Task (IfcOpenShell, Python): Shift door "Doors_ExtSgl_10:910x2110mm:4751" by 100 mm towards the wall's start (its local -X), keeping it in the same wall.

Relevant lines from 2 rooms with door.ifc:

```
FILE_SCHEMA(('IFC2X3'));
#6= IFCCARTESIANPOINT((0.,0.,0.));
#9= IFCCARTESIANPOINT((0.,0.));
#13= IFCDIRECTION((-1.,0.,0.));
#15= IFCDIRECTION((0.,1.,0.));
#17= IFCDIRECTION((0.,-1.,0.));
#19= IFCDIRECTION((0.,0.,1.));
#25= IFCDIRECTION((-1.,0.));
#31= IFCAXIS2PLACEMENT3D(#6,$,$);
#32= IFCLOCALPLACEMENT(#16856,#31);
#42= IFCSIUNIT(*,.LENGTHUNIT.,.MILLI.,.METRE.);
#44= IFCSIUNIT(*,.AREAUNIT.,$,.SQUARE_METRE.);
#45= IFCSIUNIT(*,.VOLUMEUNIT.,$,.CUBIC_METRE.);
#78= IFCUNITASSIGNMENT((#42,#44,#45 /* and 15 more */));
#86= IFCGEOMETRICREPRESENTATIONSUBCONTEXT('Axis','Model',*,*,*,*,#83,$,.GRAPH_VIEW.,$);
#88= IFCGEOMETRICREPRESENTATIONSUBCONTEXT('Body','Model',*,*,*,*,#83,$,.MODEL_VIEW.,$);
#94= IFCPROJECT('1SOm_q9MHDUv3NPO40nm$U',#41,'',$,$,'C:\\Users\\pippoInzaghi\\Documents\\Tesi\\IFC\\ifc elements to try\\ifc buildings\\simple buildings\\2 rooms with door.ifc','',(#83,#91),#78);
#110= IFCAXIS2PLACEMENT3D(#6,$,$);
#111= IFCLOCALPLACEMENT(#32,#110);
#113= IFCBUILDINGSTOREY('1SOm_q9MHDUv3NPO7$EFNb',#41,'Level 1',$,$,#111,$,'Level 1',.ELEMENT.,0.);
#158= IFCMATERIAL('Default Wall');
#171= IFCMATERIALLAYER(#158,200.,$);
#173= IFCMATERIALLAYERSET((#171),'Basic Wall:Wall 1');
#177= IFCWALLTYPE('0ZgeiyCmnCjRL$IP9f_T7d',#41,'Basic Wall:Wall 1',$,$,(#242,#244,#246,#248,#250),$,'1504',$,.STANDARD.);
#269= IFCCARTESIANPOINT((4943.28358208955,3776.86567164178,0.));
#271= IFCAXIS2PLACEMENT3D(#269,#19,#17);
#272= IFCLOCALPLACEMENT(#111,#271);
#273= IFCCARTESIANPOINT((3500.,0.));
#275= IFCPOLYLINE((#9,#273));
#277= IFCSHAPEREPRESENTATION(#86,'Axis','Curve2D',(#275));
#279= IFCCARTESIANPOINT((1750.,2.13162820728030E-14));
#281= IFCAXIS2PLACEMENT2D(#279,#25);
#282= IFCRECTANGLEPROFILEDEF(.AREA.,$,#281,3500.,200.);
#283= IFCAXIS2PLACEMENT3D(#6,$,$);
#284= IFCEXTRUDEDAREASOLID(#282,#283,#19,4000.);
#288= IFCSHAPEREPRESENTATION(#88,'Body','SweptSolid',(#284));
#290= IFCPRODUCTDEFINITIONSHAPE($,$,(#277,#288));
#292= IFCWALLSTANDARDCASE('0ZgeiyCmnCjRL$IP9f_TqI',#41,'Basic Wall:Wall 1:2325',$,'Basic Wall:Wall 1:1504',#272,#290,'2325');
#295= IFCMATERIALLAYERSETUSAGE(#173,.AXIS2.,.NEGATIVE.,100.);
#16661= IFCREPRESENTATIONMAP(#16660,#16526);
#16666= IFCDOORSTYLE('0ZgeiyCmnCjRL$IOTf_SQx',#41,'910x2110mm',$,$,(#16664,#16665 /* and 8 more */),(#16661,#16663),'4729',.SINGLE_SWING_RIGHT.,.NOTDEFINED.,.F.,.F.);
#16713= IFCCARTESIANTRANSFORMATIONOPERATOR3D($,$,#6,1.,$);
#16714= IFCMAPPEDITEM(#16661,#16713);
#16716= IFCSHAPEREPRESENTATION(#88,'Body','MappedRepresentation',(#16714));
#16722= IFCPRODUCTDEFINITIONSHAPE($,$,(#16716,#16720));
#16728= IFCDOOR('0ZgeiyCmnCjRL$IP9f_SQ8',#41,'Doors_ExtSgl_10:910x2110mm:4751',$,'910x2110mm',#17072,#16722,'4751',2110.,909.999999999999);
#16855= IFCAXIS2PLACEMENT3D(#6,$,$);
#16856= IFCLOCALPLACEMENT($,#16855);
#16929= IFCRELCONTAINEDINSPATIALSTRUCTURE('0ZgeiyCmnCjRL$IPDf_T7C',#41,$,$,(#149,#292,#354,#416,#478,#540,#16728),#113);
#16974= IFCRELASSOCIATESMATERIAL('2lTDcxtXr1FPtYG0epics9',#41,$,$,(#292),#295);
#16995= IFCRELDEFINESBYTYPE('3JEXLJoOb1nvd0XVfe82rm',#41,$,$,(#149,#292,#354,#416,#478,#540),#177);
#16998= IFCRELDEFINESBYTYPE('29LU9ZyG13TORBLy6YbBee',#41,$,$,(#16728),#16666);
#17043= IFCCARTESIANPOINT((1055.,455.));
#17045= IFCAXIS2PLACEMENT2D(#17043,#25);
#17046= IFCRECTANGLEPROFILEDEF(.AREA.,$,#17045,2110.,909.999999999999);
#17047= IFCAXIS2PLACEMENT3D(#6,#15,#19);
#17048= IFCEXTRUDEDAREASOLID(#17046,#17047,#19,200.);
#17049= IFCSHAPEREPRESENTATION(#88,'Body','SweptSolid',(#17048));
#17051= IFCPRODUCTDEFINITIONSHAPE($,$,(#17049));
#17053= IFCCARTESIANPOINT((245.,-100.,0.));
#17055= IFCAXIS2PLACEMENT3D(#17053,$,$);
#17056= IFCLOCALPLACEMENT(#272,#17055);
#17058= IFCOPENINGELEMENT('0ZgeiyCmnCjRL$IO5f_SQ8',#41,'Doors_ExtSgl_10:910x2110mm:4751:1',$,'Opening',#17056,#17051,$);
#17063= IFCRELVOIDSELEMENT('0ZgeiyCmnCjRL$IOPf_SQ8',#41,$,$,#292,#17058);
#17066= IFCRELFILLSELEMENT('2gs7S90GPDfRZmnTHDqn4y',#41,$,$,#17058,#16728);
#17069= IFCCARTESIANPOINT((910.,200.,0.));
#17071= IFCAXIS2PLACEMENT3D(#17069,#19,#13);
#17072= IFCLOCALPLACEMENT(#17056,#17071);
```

```python
import ifcopenshell
import ifcopenshell.api.geometry
import ifcopenshell.util.placement
import ifcopenshell.util.unit

model = ifcopenshell.open("2 rooms with door.ifc")
unit_scale = ifcopenshell.util.unit.calculate_unit_scale(model)

door = model.by_id(16728)
opening = door.FillsVoids[0].RelatingOpeningElement
wall = opening.VoidsElements[0].RelatingBuildingElement

wall_matrix = ifcopenshell.util.placement.get_local_placement(wall.ObjectPlacement)
shift = wall_matrix[:3, 0] * -0.1 / unit_scale
before = ifcopenshell.util.placement.get_local_placement(door.ObjectPlacement)[:3, 3].copy()

# The door is placed relative to its opening, so it follows when the opening moves.
matrix = ifcopenshell.util.placement.get_local_placement(opening.ObjectPlacement)
matrix[:3, 3] += shift
ifcopenshell.api.geometry.edit_object_placement(
    model, product=opening, matrix=matrix, is_si=False, should_transform_children=True
)

after = ifcopenshell.util.placement.get_local_placement(door.ObjectPlacement)[:3, 3]
print("door moved by", (after - before).round(3) + 0.0)

model.write("2 rooms with door-out.ifc")
```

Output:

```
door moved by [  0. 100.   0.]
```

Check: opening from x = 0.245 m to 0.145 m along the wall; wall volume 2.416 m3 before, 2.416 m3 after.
